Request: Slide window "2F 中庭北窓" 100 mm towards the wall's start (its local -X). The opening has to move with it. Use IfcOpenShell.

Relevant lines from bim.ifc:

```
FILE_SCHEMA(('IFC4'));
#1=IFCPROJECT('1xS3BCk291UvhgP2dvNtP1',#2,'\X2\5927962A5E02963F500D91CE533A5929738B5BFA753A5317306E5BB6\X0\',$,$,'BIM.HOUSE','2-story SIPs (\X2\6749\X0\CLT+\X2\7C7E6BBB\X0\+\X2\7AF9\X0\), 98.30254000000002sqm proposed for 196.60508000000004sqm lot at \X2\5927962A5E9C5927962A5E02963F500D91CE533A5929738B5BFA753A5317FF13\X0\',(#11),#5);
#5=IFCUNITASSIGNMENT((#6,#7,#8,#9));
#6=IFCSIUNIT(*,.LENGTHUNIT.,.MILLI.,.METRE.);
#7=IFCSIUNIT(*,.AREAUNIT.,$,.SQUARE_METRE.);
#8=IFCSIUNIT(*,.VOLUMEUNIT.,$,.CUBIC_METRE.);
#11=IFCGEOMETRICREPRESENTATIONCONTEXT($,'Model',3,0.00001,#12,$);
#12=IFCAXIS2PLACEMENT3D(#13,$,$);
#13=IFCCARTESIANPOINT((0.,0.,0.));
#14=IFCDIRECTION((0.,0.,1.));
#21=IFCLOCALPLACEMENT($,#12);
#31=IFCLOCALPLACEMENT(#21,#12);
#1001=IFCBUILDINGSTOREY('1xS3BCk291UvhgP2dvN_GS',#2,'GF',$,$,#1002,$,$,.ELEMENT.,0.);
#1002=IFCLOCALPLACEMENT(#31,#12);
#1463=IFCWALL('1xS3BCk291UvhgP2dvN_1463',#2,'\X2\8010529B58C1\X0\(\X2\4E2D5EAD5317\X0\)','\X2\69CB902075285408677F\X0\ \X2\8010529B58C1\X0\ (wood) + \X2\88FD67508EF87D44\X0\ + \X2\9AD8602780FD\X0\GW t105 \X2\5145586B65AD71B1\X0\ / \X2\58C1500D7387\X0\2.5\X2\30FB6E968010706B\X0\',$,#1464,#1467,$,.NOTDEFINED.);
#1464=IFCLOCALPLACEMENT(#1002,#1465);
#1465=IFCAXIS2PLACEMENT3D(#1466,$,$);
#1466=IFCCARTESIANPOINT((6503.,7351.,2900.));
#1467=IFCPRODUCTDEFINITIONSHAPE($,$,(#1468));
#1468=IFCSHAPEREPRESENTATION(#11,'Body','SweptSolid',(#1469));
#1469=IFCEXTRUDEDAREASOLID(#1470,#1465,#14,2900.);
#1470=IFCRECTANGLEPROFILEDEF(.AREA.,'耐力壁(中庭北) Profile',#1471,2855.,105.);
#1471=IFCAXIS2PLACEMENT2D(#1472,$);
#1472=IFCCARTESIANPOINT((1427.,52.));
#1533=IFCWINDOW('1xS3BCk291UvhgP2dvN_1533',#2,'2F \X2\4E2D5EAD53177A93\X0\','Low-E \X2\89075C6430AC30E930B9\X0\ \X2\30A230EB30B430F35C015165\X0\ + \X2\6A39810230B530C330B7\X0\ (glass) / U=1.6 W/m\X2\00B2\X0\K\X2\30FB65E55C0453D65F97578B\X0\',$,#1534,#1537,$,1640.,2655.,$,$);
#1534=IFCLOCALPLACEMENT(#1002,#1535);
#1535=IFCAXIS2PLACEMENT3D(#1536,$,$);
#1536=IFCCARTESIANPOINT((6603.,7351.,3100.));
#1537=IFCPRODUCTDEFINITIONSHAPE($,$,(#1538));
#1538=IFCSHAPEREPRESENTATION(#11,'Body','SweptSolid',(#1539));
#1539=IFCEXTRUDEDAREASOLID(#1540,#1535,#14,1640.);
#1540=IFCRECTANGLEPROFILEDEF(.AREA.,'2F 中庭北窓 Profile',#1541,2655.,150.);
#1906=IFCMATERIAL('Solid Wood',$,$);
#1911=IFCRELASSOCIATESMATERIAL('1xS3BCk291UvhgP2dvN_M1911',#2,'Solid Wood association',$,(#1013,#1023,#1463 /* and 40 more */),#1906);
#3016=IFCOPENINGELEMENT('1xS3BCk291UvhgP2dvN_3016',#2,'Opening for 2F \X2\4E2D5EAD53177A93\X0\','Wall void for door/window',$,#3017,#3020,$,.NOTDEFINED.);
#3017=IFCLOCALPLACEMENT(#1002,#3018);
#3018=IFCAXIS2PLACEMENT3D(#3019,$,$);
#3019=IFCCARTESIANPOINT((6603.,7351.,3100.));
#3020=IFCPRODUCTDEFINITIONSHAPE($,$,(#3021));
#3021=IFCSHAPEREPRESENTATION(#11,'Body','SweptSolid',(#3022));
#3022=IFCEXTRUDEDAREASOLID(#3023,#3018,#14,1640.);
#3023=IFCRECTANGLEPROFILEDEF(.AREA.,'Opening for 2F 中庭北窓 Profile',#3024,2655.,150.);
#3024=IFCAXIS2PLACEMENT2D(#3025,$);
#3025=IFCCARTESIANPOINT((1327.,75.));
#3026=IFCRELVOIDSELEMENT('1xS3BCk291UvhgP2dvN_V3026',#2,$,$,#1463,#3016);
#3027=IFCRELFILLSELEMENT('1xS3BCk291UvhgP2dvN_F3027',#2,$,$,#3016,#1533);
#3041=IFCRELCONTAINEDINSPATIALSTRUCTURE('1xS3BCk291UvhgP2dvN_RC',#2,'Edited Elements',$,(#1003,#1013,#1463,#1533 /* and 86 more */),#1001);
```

```python
import ifcopenshell
import ifcopenshell.api.geometry
import ifcopenshell.util.placement
import ifcopenshell.util.unit

model = ifcopenshell.open("bim.ifc")
unit_scale = ifcopenshell.util.unit.calculate_unit_scale(model)

window = model.by_guid("1xS3BCk291UvhgP2dvN_1533")
opening = window.FillsVoids[0].RelatingOpeningElement
wall = opening.VoidsElements[0].RelatingBuildingElement

wall_matrix = ifcopenshell.util.placement.get_local_placement(wall.ObjectPlacement)
shift = wall_matrix[:3, 0] * -0.1 / unit_scale
before = ifcopenshell.util.placement.get_local_placement(window.ObjectPlacement)[:3, 3].copy()

# The window is not placed relative to its opening, so move both.
for product in (opening, window):
    matrix = ifcopenshell.util.placement.get_local_placement(product.ObjectPlacement)
    matrix[:3, 3] += shift
    ifcopenshell.api.geometry.edit_object_placement(model, product=product, matrix=matrix, is_si=False)

after = ifcopenshell.util.placement.get_local_placement(window.ObjectPlacement)[:3, 3]
print("window moved by", (after - before).round(3) + 0.0)

model.write("bim-out.ifc")
```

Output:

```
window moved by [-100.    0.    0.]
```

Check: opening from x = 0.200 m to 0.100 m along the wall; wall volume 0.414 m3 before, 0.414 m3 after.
